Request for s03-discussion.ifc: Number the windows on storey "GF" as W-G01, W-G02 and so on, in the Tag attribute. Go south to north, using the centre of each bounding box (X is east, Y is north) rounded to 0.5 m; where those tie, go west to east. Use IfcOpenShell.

First a look at what the model holds.

```python
import ifcopenshell
import ifcopenshell.util.element
import ifcopenshell.util.placement

model = ifcopenshell.open("s03-discussion.ifc")
print(model.schema)
storey = next(s for s in model.by_type("IfcBuildingStorey") if s.Name == "GF")
windows = [e for e in ifcopenshell.util.element.get_decomposition(storey) if e.is_a("IfcWindow")]
for e in sorted(windows, key=lambda e: e.id()):
    origin = ifcopenshell.util.placement.get_local_placement(e.ObjectPlacement)[:3, 3]
    print(e.id(), e.Tag, e.Name, origin.round(2) + 0.0, sep=" | ")
```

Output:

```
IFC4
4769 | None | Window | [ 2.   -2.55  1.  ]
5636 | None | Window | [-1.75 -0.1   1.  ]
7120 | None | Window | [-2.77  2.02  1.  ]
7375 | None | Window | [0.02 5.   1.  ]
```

```python
import ifcopenshell
import ifcopenshell.geom
import ifcopenshell.util.element
import ifcopenshell.util.shape

model = ifcopenshell.open("s03-discussion.ifc")
settings = ifcopenshell.geom.settings()
settings.set("use-world-coords", True)


def centre(element):
    shape = ifcopenshell.geom.create_shape(settings, element)
    return ifcopenshell.util.shape.get_bbox_centroid(shape.geometry)


storey = next(s for s in model.by_type("IfcBuildingStorey") if s.Name == "GF")
windows = [e for e in ifcopenshell.util.element.get_decomposition(storey) if e.is_a("IfcWindow")]

# Insertion points can sit at a corner or the storey origin, so sort by the geometry (in metres).
centres = {e: centre(e) for e in windows}
windows.sort(key=lambda e: (round(centres[e][1] / 0.5), centres[e][0]))

for i, e in enumerate(windows, start=1):
    number = f"W-G{i:02d}"
    e.Tag = number
    print(e.id(), number)

model.write("s03-discussion_updated.ifc")
```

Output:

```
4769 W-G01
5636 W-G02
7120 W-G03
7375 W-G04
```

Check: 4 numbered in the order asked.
